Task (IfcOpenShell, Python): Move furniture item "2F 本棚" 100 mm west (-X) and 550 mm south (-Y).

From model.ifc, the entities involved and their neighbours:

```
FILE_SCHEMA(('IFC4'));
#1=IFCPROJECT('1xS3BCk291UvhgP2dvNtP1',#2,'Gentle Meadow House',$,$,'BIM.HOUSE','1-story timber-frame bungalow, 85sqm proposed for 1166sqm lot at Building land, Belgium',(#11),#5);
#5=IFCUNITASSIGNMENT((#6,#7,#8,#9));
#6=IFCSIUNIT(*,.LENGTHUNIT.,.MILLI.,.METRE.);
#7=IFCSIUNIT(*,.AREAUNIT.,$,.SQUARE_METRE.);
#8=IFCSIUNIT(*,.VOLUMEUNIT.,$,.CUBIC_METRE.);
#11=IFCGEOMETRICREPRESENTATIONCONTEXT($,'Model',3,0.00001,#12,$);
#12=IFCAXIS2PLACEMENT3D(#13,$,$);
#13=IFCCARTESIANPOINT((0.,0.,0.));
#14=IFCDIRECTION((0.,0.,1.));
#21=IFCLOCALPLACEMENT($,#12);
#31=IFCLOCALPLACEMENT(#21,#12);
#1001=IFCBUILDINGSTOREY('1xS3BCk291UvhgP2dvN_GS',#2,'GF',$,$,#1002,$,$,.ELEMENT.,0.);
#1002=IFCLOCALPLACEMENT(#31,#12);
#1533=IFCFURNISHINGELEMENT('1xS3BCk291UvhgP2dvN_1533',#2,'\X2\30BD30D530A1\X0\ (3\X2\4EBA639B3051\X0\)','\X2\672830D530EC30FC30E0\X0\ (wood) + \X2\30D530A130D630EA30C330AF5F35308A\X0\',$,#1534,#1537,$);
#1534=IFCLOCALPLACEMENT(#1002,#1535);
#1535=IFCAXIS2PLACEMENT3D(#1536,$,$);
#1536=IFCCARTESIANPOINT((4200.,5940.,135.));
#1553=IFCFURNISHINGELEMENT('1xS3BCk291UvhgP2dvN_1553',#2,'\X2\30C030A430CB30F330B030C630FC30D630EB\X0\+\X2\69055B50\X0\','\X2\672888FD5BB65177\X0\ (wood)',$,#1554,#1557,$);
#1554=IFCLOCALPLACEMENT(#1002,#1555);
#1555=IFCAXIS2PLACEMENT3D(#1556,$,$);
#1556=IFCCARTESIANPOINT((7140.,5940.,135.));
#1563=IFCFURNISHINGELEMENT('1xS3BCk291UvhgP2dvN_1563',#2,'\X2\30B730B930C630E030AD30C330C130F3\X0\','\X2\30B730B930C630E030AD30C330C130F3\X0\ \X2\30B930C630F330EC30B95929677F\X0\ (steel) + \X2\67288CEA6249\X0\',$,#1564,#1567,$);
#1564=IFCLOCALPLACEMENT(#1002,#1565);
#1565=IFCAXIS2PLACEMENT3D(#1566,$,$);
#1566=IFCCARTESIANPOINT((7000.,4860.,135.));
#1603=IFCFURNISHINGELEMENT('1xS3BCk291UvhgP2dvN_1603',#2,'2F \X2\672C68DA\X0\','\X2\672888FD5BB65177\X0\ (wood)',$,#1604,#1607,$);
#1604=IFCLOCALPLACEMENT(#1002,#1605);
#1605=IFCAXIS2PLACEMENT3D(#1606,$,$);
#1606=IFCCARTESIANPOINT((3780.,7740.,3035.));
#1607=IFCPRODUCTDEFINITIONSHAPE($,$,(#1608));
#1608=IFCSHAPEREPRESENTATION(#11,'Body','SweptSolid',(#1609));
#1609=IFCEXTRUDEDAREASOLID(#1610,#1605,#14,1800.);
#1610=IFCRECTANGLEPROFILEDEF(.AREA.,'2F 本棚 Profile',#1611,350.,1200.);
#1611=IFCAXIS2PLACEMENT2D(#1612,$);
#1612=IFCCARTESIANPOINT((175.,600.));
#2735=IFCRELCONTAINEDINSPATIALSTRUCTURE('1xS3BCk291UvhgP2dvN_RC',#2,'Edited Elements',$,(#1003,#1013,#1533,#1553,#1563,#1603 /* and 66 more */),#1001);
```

```python
import ifcopenshell
import ifcopenshell.api.geometry
import ifcopenshell.util.placement
import ifcopenshell.util.unit

model = ifcopenshell.open("model.ifc")
unit_scale = ifcopenshell.util.unit.calculate_unit_scale(model)

item = model.by_guid("1xS3BCk291UvhgP2dvN_1603")
matrix = ifcopenshell.util.placement.get_local_placement(item.ObjectPlacement)
matrix[0, 3] -= 0.1 / unit_scale
matrix[1, 3] -= 0.55 / unit_scale
ifcopenshell.api.geometry.edit_object_placement(model, product=item, matrix=matrix, is_si=False)

print(ifcopenshell.util.placement.get_local_placement(item.ObjectPlacement).round(3) + 0.0)

model.write("model_v2.ifc")
```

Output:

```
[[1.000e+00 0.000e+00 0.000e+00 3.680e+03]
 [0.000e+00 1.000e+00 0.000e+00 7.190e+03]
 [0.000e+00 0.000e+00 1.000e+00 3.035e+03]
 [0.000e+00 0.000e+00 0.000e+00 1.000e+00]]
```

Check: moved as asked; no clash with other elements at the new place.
